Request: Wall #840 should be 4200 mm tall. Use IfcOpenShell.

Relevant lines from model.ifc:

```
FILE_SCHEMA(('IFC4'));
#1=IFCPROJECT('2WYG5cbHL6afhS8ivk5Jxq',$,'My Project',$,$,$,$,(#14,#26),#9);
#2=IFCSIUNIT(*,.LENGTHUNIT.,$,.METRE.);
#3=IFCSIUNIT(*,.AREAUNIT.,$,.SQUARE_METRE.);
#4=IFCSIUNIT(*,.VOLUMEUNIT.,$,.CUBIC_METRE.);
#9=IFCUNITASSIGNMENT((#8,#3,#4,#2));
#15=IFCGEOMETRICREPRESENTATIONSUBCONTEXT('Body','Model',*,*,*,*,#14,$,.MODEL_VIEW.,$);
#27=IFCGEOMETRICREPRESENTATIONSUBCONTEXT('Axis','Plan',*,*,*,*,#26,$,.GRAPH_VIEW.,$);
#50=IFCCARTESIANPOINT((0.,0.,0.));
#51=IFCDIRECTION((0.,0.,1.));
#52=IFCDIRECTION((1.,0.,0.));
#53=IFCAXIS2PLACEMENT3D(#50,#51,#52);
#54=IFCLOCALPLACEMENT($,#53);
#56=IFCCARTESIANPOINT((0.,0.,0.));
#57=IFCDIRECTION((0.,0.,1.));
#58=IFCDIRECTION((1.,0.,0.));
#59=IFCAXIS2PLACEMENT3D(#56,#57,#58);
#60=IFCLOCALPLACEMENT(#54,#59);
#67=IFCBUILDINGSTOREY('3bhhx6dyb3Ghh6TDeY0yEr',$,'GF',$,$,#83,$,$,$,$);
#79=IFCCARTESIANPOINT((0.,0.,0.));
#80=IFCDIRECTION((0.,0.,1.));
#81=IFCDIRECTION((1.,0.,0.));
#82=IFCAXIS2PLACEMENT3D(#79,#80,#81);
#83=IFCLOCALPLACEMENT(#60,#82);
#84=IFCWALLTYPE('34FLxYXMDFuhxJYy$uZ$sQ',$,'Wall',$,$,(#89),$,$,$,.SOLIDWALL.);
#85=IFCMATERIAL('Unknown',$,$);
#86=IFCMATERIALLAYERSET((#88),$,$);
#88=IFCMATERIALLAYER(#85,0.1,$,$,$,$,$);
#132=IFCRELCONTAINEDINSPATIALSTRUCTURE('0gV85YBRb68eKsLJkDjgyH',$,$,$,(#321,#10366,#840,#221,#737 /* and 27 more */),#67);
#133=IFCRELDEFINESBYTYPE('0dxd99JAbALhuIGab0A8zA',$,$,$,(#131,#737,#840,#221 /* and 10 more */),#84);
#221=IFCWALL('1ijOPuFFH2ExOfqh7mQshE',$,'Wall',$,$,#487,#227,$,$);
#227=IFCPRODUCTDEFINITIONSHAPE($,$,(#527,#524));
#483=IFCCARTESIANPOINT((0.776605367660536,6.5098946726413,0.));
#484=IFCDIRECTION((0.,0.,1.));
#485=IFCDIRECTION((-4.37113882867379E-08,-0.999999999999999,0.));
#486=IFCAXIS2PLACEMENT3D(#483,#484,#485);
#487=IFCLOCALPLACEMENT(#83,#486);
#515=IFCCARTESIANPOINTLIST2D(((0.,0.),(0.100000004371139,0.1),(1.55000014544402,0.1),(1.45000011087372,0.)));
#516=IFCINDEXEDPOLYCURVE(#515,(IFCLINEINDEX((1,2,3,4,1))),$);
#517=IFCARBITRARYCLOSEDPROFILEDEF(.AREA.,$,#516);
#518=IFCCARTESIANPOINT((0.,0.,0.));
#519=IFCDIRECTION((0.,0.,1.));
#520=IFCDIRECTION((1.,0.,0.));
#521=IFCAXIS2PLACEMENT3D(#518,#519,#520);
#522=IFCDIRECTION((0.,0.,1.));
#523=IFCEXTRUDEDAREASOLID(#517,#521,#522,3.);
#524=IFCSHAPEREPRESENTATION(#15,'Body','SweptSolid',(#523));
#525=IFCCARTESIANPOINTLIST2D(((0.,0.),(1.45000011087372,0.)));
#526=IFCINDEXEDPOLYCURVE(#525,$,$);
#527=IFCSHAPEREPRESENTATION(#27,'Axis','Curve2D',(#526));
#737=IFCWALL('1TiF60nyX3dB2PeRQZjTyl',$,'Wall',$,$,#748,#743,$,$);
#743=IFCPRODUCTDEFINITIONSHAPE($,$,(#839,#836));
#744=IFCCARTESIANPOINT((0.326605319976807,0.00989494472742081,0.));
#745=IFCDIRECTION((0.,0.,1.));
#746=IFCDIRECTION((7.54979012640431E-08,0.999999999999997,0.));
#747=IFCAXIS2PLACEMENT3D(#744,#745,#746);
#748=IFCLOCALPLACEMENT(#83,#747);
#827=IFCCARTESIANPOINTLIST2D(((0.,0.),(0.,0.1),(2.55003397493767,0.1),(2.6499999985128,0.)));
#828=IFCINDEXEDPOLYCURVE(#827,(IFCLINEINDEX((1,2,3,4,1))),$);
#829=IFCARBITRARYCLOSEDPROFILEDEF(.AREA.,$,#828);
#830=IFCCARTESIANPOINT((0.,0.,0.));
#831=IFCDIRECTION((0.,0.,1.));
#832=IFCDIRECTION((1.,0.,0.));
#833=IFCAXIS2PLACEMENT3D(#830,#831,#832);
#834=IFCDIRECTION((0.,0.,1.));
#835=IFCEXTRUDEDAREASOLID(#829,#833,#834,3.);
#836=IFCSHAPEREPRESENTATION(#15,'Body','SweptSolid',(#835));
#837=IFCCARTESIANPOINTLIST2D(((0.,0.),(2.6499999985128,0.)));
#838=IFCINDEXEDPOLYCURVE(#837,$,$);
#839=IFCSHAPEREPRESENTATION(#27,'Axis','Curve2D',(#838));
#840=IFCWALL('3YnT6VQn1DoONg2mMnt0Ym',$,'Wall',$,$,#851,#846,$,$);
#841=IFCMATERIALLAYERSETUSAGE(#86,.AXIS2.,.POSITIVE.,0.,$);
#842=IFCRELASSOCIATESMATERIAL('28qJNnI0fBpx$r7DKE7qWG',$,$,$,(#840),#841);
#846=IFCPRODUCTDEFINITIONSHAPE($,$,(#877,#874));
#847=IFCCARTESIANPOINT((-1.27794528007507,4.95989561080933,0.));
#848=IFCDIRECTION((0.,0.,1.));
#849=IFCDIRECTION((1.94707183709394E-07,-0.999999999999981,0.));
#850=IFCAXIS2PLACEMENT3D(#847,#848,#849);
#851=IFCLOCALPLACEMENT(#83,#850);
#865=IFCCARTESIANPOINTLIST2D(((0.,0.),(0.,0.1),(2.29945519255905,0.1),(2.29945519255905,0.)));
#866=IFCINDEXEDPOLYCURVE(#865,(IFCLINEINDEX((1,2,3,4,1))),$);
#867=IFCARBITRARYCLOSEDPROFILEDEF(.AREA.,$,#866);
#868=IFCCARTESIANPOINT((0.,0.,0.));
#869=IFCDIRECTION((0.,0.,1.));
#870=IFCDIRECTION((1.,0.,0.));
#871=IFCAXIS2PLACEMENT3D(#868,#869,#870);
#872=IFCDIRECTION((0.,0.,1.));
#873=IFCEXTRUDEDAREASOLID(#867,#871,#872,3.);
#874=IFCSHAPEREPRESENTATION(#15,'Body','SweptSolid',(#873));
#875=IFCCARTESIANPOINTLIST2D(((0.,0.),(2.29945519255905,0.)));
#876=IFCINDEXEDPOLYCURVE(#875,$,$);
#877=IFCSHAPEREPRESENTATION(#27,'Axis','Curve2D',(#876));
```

```python
import ifcopenshell
import ifcopenshell.geom
import ifcopenshell.util.representation
import ifcopenshell.util.shape
import ifcopenshell.util.unit

model = ifcopenshell.open("model.ifc")
unit_scale = ifcopenshell.util.unit.calculate_unit_scale(model)
settings = ifcopenshell.geom.settings()


def volume(element):
    """Net volume in cubic metres, openings subtracted."""
    shape = ifcopenshell.geom.create_shape(settings, element)
    return ifcopenshell.util.shape.get_volume(shape.geometry)


wall = model.by_guid("3YnT6VQn1DoONg2mMnt0Ym")
before = volume(wall)

body = ifcopenshell.util.representation.get_representation(wall, "Model", "Body")
solid = body.Items[0]
old_height = solid.Depth
solid.Depth = 4.2 / unit_scale
after = volume(wall)

print(f"height {old_height:g} -> {solid.Depth:g}, volume {before:.3f} -> {after:.3f} m3")

model.write("model_v2.ifc")
```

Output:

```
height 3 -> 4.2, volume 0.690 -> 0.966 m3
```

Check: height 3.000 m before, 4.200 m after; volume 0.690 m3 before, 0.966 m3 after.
